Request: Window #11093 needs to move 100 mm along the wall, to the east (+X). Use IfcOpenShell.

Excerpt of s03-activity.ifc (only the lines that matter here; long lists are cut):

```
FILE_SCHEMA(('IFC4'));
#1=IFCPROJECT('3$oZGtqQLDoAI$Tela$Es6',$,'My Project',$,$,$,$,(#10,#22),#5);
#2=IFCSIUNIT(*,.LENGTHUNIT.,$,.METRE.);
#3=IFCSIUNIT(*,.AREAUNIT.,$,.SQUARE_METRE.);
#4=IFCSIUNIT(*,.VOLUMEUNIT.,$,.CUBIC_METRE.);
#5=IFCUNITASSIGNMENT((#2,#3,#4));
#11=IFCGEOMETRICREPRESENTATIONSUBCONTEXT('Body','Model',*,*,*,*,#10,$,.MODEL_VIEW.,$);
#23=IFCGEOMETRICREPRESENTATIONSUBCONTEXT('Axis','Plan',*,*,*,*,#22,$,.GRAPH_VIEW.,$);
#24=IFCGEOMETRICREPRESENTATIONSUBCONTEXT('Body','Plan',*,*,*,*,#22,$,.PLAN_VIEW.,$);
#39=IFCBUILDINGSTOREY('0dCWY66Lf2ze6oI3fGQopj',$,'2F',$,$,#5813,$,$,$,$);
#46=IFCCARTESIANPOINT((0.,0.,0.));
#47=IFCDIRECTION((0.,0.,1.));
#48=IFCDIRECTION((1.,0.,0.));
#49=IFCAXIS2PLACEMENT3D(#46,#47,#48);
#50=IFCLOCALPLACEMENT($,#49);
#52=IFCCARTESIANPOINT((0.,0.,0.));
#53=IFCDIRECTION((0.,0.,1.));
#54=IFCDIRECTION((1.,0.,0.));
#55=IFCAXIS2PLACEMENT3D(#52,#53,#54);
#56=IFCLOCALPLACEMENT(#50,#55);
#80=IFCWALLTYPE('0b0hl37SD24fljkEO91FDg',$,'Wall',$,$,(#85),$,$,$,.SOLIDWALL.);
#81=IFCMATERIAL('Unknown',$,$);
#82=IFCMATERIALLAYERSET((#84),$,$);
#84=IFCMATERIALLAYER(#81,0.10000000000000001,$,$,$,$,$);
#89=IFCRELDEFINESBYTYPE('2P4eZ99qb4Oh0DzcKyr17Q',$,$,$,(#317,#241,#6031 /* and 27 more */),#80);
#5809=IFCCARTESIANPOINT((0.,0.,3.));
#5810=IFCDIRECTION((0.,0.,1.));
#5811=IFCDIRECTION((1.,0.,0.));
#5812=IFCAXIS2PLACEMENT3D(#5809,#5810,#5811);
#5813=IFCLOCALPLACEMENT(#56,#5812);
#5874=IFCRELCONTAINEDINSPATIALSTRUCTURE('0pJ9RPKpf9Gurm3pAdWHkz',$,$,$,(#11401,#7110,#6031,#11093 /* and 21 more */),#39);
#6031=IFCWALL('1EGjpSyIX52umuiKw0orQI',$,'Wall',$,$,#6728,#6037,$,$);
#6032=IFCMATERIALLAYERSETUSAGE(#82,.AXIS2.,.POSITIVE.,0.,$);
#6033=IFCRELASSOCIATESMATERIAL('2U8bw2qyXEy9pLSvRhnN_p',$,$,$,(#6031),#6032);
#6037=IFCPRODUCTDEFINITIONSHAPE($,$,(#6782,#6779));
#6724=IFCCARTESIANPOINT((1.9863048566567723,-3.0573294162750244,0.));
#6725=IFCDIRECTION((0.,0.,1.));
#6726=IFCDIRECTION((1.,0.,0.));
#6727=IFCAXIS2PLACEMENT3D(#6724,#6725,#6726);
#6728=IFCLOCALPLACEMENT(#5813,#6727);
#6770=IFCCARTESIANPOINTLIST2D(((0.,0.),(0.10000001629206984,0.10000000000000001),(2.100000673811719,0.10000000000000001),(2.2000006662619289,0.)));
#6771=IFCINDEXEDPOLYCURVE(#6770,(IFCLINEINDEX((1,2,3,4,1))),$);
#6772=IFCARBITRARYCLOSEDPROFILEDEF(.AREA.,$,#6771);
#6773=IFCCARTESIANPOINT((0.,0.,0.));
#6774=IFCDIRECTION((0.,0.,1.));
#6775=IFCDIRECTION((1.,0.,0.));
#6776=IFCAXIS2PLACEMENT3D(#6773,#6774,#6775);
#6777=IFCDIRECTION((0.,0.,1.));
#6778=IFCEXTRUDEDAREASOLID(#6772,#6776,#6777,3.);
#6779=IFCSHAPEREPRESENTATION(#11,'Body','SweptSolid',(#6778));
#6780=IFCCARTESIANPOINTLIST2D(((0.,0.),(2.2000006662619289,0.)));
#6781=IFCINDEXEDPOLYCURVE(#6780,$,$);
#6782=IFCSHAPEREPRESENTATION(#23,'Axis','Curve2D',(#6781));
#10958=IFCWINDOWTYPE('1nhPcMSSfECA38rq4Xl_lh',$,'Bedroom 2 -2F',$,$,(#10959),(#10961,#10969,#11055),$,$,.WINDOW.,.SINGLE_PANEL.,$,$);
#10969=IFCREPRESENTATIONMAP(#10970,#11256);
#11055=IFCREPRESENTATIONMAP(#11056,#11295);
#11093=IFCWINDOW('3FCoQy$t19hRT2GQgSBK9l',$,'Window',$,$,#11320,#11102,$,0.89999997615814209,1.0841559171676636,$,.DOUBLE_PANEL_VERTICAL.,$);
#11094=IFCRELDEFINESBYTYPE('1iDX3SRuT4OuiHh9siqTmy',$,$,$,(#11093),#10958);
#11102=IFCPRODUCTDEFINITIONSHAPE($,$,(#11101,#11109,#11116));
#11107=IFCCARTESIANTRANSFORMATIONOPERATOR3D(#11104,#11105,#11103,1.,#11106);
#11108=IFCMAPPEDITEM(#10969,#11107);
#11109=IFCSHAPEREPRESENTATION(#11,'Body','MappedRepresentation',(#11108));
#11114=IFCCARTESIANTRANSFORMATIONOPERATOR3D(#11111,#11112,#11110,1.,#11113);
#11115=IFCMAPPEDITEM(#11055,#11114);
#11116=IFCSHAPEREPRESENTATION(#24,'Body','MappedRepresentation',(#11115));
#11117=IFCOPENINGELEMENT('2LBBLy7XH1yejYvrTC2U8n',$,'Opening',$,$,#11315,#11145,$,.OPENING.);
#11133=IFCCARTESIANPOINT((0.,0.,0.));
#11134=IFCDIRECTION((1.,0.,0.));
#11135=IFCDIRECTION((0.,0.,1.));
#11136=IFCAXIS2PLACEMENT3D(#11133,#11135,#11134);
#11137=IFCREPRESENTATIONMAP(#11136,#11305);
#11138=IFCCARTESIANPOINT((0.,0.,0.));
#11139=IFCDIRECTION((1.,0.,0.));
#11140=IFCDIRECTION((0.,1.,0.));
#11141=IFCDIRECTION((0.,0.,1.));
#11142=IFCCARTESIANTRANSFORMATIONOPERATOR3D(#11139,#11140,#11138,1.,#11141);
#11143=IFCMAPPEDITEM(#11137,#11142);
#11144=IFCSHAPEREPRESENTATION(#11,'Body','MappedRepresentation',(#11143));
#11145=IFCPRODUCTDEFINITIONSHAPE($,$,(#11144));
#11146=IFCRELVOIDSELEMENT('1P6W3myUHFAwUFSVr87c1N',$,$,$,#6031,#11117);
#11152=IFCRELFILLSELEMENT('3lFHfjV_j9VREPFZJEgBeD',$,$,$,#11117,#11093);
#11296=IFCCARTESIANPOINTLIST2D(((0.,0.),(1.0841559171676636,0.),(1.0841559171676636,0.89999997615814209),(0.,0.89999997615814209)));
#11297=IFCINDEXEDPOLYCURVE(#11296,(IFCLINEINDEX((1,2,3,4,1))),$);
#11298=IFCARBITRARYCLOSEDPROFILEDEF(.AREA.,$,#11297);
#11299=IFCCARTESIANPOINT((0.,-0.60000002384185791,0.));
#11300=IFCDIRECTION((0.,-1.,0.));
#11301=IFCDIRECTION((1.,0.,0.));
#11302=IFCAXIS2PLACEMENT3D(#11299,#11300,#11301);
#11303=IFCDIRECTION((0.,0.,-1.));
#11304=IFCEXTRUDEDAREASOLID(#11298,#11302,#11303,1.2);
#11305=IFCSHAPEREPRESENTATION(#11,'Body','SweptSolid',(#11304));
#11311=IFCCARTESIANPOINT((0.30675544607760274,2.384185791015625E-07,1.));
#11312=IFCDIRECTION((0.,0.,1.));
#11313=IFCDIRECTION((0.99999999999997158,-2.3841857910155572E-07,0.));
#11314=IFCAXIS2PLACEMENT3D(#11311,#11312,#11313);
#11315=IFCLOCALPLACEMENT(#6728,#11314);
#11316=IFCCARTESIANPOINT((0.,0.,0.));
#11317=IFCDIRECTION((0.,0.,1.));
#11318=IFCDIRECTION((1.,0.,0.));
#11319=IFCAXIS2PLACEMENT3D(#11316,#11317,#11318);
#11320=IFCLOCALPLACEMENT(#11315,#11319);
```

```python
import ifcopenshell
import ifcopenshell.api.geometry
import ifcopenshell.util.placement

model = ifcopenshell.open("s03-activity.ifc")

window = model.by_id(11093)
opening = window.FillsVoids[0].RelatingOpeningElement
wall = opening.VoidsElements[0].RelatingBuildingElement

wall_matrix = ifcopenshell.util.placement.get_local_placement(wall.ObjectPlacement)
shift = wall_matrix[:3, 0] * 0.1
before = ifcopenshell.util.placement.get_local_placement(window.ObjectPlacement)[:3, 3].copy()

# The window is placed relative to its opening, so it follows when the opening moves.
matrix = ifcopenshell.util.placement.get_local_placement(opening.ObjectPlacement)
matrix[:3, 3] += shift
ifcopenshell.api.geometry.edit_object_placement(
    model, product=opening, matrix=matrix, is_si=False, should_transform_children=True
)

after = ifcopenshell.util.placement.get_local_placement(window.ObjectPlacement)[:3, 3]
print("window moved by", (after - before).round(3) + 0.0)

model.write("s03-activity_rev.ifc")
```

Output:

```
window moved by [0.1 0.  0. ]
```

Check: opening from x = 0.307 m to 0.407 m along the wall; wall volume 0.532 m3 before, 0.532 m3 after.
